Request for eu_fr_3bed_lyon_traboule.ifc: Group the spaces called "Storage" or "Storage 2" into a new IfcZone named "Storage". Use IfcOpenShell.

First a look at what the model holds.

```python
import ifcopenshell

model = ifcopenshell.open("eu_fr_3bed_lyon_traboule.ifc")
print(model.schema)
seen = {}
for space in model.by_type("IfcSpace"):
    seen[space.LongName] = seen.get(space.LongName, 0) + 1
for name, count in sorted(seen.items(), key=str):
    print(count, "x", name)
print("zones:", [z.Name for z in model.by_type("IfcZone")][:20])
```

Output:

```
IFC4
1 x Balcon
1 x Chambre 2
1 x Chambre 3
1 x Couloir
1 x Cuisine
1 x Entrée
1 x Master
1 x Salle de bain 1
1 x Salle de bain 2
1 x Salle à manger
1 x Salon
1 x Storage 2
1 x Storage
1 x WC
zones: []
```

```python
import ifcopenshell
import ifcopenshell.api.group
import ifcopenshell.api.root

model = ifcopenshell.open("eu_fr_3bed_lyon_traboule.ifc")

names = {"Storage", "Storage 2"}
spaces = [s for s in model.by_type("IfcSpace") if s.LongName in names]

zone = ifcopenshell.api.root.create_entity(model, ifc_class="IfcZone", name="Storage")
ifcopenshell.api.group.assign_group(model, products=spaces, group=zone)
print(len(spaces), "spaces in", zone.Name)

model.write("eu_fr_3bed_lyon_traboule-out.ifc")
```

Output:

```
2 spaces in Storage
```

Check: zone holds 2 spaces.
